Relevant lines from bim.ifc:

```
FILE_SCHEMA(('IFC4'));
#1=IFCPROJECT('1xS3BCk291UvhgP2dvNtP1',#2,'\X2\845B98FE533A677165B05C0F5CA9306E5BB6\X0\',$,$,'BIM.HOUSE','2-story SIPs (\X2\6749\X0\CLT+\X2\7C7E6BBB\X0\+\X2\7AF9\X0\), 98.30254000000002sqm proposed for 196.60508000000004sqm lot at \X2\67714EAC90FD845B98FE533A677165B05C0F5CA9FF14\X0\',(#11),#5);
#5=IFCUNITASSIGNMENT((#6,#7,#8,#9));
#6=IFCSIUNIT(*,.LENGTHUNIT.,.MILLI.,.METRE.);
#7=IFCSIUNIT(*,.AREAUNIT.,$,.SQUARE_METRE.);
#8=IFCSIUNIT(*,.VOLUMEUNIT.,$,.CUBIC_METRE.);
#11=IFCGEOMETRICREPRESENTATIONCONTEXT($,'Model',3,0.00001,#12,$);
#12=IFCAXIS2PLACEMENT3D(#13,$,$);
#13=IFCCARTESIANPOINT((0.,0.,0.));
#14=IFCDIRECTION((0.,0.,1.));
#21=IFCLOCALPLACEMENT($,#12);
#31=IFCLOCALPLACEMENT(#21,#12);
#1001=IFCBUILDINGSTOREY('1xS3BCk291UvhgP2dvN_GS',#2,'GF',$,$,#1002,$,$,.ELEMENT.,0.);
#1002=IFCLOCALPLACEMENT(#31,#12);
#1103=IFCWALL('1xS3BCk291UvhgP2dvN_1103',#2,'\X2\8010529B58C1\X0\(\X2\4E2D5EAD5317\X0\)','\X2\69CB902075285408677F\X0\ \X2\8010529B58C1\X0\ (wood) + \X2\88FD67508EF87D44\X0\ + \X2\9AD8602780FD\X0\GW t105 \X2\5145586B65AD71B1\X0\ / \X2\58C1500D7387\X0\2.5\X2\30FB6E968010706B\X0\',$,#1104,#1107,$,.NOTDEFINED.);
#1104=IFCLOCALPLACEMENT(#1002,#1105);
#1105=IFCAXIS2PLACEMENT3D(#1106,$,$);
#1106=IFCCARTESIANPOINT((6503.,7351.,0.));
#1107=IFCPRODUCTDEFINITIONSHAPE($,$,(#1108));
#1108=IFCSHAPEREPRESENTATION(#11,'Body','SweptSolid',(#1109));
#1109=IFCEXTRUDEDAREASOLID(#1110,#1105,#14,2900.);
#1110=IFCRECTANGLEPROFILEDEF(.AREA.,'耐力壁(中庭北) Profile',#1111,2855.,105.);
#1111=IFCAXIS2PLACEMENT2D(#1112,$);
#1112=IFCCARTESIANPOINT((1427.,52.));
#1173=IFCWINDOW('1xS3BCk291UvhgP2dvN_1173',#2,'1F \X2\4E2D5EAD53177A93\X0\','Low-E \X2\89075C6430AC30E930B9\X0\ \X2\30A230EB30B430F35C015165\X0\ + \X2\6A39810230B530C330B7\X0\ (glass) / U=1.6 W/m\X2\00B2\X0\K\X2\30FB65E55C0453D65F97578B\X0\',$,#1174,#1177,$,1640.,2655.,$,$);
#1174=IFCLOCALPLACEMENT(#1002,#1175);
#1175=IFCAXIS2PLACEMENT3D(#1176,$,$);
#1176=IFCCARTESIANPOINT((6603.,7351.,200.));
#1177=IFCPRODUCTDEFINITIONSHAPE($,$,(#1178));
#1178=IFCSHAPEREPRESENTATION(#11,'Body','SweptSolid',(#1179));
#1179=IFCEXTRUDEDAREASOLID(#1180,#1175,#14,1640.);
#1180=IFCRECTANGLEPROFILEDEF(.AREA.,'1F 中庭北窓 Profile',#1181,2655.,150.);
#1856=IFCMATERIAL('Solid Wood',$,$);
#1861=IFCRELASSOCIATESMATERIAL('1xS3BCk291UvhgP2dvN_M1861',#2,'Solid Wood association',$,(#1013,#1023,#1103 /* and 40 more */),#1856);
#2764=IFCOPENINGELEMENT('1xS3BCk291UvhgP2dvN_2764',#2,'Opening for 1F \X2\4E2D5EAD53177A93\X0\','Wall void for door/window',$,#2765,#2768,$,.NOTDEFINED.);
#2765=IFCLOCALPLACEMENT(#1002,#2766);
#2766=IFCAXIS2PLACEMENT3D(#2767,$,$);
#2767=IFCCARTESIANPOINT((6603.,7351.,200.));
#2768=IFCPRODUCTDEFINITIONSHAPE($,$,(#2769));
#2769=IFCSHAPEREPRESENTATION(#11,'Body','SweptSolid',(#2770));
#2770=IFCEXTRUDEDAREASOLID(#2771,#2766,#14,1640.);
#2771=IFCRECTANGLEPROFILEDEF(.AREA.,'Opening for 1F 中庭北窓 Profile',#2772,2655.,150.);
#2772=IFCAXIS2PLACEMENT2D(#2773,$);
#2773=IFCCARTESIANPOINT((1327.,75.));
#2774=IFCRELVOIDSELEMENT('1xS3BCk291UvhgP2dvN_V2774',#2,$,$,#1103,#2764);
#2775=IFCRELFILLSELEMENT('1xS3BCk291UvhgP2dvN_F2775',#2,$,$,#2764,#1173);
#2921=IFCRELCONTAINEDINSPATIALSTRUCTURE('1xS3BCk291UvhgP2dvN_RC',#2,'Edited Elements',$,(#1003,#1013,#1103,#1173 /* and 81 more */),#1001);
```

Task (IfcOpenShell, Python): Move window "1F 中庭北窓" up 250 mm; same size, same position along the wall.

```python
import numpy as np
import ifcopenshell
import ifcopenshell.api.geometry
import ifcopenshell.util.placement
import ifcopenshell.util.unit

model = ifcopenshell.open("bim.ifc")
unit_scale = ifcopenshell.util.unit.calculate_unit_scale(model)

window = model.by_guid("1xS3BCk291UvhgP2dvN_1173")
opening = window.FillsVoids[0].RelatingOpeningElement
dz = 0.25 / unit_scale

shift = np.array([0.0, 0.0, dz])
# The window is not placed relative to its opening, so move both.
for product in (opening, window):
    matrix = ifcopenshell.util.placement.get_local_placement(product.ObjectPlacement)
    matrix[:3, 3] += shift
    ifcopenshell.api.geometry.edit_object_placement(model, product=product, matrix=matrix, is_si=False)

print(f"moved by {dz * unit_scale:+.3f} m")

model.write("bim_rev.ifc")
```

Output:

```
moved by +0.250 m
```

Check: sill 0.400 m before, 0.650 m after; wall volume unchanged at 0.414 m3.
